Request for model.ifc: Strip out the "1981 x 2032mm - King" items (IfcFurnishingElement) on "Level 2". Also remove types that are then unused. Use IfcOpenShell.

First a look at what the model holds.

```python
import ifcopenshell
import ifcopenshell.util.element

model = ifcopenshell.open("model.ifc")
print(model.schema)
storey = next(s for s in model.by_type("IfcBuildingStorey") if s.Name == "Level 2")
furniture = [e for e in ifcopenshell.util.element.get_decomposition(storey) if e.is_a("IfcFurnishingElement")]
seen = {}
for e in furniture:
    element_type = ifcopenshell.util.element.get_type(e)
    name = element_type.Name if element_type not in (None, e) else None
    seen[name] = seen.get(name, 0) + 1
for name, count in sorted(seen.items(), key=str):
    print(count, "x", name)
```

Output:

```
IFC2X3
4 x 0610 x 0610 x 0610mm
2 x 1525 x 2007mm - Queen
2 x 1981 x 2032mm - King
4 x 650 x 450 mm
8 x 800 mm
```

```python
import ifcopenshell
import ifcopenshell.api.root
import ifcopenshell.util.element

model = ifcopenshell.open("model.ifc")

storey = next(s for s in model.by_type("IfcBuildingStorey") if s.Name == "Level 2")
furniture = [e for e in ifcopenshell.util.element.get_decomposition(storey) if e.is_a("IfcFurnishingElement")]
targets = [e for e in furniture if (t := ifcopenshell.util.element.get_type(e)) not in (None, e) and t.Name == "1981 x 2032mm - King"]
types = {ifcopenshell.util.element.get_type(e) for e in targets} - {None, *targets}

for e in targets:
    ifcopenshell.api.root.remove_product(model, product=e)
print(len(targets), "removed")

unused = [t for t in types if not ifcopenshell.util.element.get_types(t)]
for t in unused:
    ifcopenshell.api.root.remove_product(model, product=t)
print(len(unused), "unused types removed")

model.write("model-out.ifc")
```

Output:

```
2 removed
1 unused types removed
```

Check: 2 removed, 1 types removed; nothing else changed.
